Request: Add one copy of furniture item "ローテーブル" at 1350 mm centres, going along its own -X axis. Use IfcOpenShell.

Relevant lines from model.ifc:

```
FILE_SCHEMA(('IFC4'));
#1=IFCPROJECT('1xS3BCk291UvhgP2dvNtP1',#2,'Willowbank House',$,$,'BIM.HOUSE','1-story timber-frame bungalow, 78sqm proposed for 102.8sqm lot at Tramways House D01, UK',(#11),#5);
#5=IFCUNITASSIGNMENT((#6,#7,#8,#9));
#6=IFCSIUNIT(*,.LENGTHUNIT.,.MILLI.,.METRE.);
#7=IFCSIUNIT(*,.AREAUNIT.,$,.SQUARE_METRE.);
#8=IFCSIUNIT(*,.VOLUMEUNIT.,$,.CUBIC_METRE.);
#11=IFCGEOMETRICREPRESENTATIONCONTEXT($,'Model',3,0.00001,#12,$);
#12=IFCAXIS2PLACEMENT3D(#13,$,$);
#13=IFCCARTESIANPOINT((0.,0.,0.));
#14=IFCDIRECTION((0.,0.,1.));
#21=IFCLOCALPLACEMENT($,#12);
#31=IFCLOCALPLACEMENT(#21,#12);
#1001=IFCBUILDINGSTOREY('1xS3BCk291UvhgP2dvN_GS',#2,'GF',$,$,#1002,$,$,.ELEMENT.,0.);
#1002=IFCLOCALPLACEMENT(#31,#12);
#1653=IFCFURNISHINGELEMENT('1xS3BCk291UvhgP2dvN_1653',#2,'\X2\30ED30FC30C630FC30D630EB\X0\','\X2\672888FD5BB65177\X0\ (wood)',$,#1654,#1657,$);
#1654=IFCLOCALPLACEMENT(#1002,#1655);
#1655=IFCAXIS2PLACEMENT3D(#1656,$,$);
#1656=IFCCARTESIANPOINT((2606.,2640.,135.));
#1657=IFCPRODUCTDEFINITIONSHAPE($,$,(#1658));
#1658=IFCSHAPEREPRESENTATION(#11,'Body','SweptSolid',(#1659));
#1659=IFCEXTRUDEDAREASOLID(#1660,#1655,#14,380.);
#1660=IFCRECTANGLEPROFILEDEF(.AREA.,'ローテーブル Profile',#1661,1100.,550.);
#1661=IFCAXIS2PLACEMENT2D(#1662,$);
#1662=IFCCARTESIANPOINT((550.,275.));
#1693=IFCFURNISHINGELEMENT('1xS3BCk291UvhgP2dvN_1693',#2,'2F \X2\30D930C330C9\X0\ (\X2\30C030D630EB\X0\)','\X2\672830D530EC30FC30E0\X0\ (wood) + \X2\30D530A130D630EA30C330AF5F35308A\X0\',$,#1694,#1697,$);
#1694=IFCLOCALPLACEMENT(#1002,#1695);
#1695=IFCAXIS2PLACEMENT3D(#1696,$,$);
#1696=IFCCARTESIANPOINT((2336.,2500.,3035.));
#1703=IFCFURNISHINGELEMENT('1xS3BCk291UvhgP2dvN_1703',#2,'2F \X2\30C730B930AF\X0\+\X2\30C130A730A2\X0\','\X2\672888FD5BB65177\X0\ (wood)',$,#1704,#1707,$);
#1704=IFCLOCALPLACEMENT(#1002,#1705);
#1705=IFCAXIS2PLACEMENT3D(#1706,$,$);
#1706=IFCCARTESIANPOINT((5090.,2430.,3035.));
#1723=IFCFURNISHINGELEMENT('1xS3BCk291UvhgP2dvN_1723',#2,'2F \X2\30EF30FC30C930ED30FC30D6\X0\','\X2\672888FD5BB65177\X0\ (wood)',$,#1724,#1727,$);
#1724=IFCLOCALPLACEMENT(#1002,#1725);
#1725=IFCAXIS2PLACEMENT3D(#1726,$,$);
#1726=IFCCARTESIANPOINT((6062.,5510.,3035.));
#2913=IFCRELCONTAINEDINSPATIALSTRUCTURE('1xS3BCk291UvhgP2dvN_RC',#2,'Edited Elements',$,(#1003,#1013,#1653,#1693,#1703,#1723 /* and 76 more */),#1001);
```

```python
import ifcopenshell
import ifcopenshell.api.geometry
import ifcopenshell.api.root
import ifcopenshell.util.element
import ifcopenshell.util.placement
import ifcopenshell.util.unit

model = ifcopenshell.open("model.ifc")
unit_scale = ifcopenshell.util.unit.calculate_unit_scale(model)


def reuse_history(source, copy):
    """copy_class also copies each property set's owner history, people and application; keep the originals."""
    for rel in copy.IsDefinedBy:
        if rel.is_a("IfcRelDefinesByProperties") and (history := rel.RelatingPropertyDefinition.OwnerHistory):
            rel.RelatingPropertyDefinition.OwnerHistory = source.OwnerHistory
            ifcopenshell.util.element.remove_deep2(model, history)


source = model.by_guid("1xS3BCk291UvhgP2dvN_1653")
base = ifcopenshell.util.placement.get_local_placement(source.ObjectPlacement)
step = -base[:3, 0] * 1.35 / unit_scale

for i in range(1, 2):
    copy = ifcopenshell.api.root.copy_class(model, product=source)
    copy.Representation = ifcopenshell.util.element.copy_deep(
        model, source.Representation, exclude=["IfcGeometricRepresentationContext", "IfcRepresentationMap"]
    )
    reuse_history(source, copy)
    matrix = base.copy()
    matrix[:3, 3] += i * step
    print("added at", matrix[:3, 3].round(3) + 0.0)
    ifcopenshell.api.geometry.edit_object_placement(model, product=copy, matrix=matrix, is_si=False)

model.write("model_updated.ifc")
```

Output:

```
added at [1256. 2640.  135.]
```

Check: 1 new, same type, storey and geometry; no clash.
